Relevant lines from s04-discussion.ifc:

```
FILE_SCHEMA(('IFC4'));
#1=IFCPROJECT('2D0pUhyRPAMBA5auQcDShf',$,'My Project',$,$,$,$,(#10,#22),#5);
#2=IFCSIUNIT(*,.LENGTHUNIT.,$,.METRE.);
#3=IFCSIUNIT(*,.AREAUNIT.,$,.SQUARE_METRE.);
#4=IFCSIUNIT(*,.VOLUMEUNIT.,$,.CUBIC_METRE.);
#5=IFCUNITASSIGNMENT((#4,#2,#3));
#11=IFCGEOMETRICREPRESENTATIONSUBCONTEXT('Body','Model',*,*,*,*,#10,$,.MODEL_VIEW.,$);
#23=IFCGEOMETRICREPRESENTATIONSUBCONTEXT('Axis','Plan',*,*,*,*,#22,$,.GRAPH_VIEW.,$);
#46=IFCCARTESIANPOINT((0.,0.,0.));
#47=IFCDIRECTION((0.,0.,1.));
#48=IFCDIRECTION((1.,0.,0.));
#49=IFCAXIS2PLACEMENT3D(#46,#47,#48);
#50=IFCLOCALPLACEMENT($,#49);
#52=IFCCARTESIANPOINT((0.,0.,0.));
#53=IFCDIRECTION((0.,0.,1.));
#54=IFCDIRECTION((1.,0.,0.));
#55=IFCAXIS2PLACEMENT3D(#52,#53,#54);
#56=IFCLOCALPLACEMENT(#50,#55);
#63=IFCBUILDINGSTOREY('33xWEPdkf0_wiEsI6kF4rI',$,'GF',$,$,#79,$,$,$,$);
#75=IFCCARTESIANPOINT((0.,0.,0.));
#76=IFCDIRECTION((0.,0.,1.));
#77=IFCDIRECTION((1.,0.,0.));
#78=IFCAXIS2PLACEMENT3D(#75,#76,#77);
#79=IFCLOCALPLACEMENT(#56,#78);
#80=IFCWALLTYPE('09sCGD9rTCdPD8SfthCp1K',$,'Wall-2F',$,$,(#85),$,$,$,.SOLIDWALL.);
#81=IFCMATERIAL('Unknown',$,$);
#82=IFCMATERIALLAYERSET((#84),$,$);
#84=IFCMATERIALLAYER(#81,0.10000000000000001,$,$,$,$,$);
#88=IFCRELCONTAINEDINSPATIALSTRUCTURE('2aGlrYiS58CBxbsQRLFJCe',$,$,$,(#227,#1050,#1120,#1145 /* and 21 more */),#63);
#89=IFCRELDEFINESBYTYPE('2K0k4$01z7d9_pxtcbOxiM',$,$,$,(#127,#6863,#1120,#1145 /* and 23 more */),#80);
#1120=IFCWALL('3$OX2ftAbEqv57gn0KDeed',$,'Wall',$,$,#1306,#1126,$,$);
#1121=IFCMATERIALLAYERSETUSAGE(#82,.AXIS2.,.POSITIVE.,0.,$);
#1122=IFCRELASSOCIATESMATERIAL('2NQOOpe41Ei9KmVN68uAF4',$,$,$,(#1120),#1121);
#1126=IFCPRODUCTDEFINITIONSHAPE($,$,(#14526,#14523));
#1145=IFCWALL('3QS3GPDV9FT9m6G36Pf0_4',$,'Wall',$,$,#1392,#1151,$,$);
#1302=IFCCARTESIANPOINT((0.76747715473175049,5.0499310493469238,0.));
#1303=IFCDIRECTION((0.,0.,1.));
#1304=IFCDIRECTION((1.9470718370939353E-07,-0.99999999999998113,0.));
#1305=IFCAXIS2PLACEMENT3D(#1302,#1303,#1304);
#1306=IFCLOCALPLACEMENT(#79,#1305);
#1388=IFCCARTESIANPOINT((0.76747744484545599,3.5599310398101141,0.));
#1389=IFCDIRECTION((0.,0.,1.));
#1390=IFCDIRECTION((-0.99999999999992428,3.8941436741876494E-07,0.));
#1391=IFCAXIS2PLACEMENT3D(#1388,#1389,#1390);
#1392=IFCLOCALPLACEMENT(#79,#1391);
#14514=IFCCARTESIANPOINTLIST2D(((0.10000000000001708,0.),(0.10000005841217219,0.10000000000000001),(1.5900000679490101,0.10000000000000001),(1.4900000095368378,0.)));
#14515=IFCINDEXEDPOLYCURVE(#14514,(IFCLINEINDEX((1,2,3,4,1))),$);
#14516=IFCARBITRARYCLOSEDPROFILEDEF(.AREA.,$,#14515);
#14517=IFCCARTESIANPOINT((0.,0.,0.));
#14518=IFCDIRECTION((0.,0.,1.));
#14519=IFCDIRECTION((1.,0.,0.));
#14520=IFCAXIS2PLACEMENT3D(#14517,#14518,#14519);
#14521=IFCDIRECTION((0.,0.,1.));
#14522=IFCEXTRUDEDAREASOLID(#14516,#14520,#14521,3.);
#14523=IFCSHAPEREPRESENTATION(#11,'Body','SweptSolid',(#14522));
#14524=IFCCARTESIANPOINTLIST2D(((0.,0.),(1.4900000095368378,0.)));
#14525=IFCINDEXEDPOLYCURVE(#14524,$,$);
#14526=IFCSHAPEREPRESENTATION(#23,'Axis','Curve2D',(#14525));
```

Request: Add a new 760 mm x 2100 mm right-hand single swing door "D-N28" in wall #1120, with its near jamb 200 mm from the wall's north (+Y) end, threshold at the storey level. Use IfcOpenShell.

```python
import numpy as np
import ifcopenshell
import ifcopenshell.api.feature
import ifcopenshell.api.geometry
import ifcopenshell.api.root
import ifcopenshell.api.spatial
import ifcopenshell.geom
import ifcopenshell.util.element
import ifcopenshell.util.placement
import ifcopenshell.util.representation
import ifcopenshell.util.shape
import ifcopenshell.util.unit

model = ifcopenshell.open("s04-discussion.ifc")
unit_scale = ifcopenshell.util.unit.calculate_unit_scale(model)
settings = ifcopenshell.geom.settings()


def volume(element):
    """Net volume in cubic metres, openings subtracted."""
    shape = ifcopenshell.geom.create_shape(settings, element)
    return ifcopenshell.util.shape.get_volume(shape.geometry)


wall = model.by_guid("3$OX2ftAbEqv57gn0KDeed")
storey = ifcopenshell.util.element.get_container(wall, ifc_class="IfcBuildingStorey")
context = ifcopenshell.util.representation.get_context(model, "Model", "Body", "MODEL_VIEW")
before = volume(wall)

width, height, from_end, sill = 0.76, 2.1, 0.2, 0.0  # metres

# The wall runs along its own X axis, and the end named is its -X end.
wall_shape = ifcopenshell.geom.create_shape(settings, wall)
x, y, z = ifcopenshell.util.shape.get_vertices(wall_shape.geometry).T
start = x.min() + from_end
face, thickness = float(y.min()), float(y.max() - y.min())
wall_matrix = ifcopenshell.util.placement.get_local_placement(wall.ObjectPlacement)
level = ifcopenshell.util.placement.get_local_placement(storey.ObjectPlacement)[2, 3]


def in_wall(x, y):
    """Placement at x, y metres in the wall's axes, at sill height."""
    matrix = wall_matrix.copy()
    matrix[:, 3] = wall_matrix @ np.array([x / unit_scale, y / unit_scale, 0.0, 1.0])
    matrix[2, 3] = level + sill / unit_scale
    return matrix


# Opening: a box that overshoots both wall faces by 50 mm.
opening = ifcopenshell.api.root.create_entity(model, ifc_class="IfcOpeningElement", predefined_type="OPENING")
box = ifcopenshell.api.geometry.add_wall_representation(
    model, context=context, length=width, height=height, thickness=thickness + 0.1
)
ifcopenshell.api.geometry.assign_representation(model, product=opening, representation=box)
ifcopenshell.api.geometry.edit_object_placement(model, product=opening, matrix=in_wall(start, face - 0.05), is_si=False)
ifcopenshell.api.feature.add_feature(model, feature=opening, element=wall)

door = ifcopenshell.api.root.create_entity(model, ifc_class="IfcDoor", name="D-N28", predefined_type="DOOR")
door.OverallWidth, door.OverallHeight = width / unit_scale, height / unit_scale
door.OperationType = "SINGLE_SWING_RIGHT"
body = ifcopenshell.api.geometry.add_door_representation(
    model,
    context=context,
    overall_width=door.OverallWidth,
    overall_height=door.OverallHeight,
    operation_type="SINGLE_SWING_RIGHT",
    lining_properties={"LiningDepth": thickness / unit_scale, "ThresholdDepth": thickness / unit_scale},
)
ifcopenshell.api.geometry.assign_representation(model, product=door, representation=body)
ifcopenshell.api.spatial.assign_container(model, products=[door], relating_structure=storey)
ifcopenshell.api.feature.add_filling(model, opening=opening, element=door)

# The lining spans the wall, so the door starts at the wall face.
ifcopenshell.api.geometry.edit_object_placement(model, product=door, matrix=in_wall(start, face), is_si=False)

after = volume(wall)

print(f"wall volume {before:.3f} -> {after:.3f} m3")

model.write("s04-discussion_rev.ifc")
```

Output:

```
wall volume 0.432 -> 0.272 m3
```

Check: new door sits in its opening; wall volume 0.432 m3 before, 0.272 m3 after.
